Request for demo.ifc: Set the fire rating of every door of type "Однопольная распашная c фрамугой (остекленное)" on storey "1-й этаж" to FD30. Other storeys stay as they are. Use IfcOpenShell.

First a look at what the model holds.

```python
import ifcopenshell
import ifcopenshell.util.element

model = ifcopenshell.open("demo.ifc")
print(model.schema)
storey = next(s for s in model.by_type("IfcBuildingStorey") if s.Name == "1-й этаж")
doors = [e for e in ifcopenshell.util.element.get_decomposition(storey) if e.is_a("IfcDoor")]
seen = {}
for e in doors:
    element_type = ifcopenshell.util.element.get_type(e)
    key = (element_type.Name if element_type != e and element_type else None, ifcopenshell.util.element.get_pset(e, "Pset_DoorCommon", "FireRating"))
    seen[key] = seen.get(key, 0) + 1
for (name, value), count in sorted(seen.items(), key=str):
    print(count, "x", name, "|", value)
```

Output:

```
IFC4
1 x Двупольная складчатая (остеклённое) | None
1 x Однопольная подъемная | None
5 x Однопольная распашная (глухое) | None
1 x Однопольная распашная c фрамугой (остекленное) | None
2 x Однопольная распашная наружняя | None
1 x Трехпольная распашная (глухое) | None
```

```python
import ifcopenshell
import ifcopenshell.api.pset
import ifcopenshell.util.element

model = ifcopenshell.open("demo.ifc")

storey = next(s for s in model.by_type("IfcBuildingStorey") if s.Name == "1-й этаж")
doors = [e for e in ifcopenshell.util.element.get_decomposition(storey) if e.is_a("IfcDoor")]

count = 0
for e in doors:
    element_type = ifcopenshell.util.element.get_type(e)
    if element_type in (None, e) or element_type.Name != "Однопольная распашная c фрамугой (остекленное)":
        continue
    # add_pset returns the element's existing set when there is one.
    pset = ifcopenshell.api.pset.add_pset(model, product=e, name="Pset_DoorCommon")
    ifcopenshell.api.pset.edit_pset(model, pset=pset, properties={"FireRating": "FD30"})
    count += 1

print(count, "doors updated")

model.write("demo_updated.ifc")
```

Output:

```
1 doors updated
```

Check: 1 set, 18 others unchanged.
